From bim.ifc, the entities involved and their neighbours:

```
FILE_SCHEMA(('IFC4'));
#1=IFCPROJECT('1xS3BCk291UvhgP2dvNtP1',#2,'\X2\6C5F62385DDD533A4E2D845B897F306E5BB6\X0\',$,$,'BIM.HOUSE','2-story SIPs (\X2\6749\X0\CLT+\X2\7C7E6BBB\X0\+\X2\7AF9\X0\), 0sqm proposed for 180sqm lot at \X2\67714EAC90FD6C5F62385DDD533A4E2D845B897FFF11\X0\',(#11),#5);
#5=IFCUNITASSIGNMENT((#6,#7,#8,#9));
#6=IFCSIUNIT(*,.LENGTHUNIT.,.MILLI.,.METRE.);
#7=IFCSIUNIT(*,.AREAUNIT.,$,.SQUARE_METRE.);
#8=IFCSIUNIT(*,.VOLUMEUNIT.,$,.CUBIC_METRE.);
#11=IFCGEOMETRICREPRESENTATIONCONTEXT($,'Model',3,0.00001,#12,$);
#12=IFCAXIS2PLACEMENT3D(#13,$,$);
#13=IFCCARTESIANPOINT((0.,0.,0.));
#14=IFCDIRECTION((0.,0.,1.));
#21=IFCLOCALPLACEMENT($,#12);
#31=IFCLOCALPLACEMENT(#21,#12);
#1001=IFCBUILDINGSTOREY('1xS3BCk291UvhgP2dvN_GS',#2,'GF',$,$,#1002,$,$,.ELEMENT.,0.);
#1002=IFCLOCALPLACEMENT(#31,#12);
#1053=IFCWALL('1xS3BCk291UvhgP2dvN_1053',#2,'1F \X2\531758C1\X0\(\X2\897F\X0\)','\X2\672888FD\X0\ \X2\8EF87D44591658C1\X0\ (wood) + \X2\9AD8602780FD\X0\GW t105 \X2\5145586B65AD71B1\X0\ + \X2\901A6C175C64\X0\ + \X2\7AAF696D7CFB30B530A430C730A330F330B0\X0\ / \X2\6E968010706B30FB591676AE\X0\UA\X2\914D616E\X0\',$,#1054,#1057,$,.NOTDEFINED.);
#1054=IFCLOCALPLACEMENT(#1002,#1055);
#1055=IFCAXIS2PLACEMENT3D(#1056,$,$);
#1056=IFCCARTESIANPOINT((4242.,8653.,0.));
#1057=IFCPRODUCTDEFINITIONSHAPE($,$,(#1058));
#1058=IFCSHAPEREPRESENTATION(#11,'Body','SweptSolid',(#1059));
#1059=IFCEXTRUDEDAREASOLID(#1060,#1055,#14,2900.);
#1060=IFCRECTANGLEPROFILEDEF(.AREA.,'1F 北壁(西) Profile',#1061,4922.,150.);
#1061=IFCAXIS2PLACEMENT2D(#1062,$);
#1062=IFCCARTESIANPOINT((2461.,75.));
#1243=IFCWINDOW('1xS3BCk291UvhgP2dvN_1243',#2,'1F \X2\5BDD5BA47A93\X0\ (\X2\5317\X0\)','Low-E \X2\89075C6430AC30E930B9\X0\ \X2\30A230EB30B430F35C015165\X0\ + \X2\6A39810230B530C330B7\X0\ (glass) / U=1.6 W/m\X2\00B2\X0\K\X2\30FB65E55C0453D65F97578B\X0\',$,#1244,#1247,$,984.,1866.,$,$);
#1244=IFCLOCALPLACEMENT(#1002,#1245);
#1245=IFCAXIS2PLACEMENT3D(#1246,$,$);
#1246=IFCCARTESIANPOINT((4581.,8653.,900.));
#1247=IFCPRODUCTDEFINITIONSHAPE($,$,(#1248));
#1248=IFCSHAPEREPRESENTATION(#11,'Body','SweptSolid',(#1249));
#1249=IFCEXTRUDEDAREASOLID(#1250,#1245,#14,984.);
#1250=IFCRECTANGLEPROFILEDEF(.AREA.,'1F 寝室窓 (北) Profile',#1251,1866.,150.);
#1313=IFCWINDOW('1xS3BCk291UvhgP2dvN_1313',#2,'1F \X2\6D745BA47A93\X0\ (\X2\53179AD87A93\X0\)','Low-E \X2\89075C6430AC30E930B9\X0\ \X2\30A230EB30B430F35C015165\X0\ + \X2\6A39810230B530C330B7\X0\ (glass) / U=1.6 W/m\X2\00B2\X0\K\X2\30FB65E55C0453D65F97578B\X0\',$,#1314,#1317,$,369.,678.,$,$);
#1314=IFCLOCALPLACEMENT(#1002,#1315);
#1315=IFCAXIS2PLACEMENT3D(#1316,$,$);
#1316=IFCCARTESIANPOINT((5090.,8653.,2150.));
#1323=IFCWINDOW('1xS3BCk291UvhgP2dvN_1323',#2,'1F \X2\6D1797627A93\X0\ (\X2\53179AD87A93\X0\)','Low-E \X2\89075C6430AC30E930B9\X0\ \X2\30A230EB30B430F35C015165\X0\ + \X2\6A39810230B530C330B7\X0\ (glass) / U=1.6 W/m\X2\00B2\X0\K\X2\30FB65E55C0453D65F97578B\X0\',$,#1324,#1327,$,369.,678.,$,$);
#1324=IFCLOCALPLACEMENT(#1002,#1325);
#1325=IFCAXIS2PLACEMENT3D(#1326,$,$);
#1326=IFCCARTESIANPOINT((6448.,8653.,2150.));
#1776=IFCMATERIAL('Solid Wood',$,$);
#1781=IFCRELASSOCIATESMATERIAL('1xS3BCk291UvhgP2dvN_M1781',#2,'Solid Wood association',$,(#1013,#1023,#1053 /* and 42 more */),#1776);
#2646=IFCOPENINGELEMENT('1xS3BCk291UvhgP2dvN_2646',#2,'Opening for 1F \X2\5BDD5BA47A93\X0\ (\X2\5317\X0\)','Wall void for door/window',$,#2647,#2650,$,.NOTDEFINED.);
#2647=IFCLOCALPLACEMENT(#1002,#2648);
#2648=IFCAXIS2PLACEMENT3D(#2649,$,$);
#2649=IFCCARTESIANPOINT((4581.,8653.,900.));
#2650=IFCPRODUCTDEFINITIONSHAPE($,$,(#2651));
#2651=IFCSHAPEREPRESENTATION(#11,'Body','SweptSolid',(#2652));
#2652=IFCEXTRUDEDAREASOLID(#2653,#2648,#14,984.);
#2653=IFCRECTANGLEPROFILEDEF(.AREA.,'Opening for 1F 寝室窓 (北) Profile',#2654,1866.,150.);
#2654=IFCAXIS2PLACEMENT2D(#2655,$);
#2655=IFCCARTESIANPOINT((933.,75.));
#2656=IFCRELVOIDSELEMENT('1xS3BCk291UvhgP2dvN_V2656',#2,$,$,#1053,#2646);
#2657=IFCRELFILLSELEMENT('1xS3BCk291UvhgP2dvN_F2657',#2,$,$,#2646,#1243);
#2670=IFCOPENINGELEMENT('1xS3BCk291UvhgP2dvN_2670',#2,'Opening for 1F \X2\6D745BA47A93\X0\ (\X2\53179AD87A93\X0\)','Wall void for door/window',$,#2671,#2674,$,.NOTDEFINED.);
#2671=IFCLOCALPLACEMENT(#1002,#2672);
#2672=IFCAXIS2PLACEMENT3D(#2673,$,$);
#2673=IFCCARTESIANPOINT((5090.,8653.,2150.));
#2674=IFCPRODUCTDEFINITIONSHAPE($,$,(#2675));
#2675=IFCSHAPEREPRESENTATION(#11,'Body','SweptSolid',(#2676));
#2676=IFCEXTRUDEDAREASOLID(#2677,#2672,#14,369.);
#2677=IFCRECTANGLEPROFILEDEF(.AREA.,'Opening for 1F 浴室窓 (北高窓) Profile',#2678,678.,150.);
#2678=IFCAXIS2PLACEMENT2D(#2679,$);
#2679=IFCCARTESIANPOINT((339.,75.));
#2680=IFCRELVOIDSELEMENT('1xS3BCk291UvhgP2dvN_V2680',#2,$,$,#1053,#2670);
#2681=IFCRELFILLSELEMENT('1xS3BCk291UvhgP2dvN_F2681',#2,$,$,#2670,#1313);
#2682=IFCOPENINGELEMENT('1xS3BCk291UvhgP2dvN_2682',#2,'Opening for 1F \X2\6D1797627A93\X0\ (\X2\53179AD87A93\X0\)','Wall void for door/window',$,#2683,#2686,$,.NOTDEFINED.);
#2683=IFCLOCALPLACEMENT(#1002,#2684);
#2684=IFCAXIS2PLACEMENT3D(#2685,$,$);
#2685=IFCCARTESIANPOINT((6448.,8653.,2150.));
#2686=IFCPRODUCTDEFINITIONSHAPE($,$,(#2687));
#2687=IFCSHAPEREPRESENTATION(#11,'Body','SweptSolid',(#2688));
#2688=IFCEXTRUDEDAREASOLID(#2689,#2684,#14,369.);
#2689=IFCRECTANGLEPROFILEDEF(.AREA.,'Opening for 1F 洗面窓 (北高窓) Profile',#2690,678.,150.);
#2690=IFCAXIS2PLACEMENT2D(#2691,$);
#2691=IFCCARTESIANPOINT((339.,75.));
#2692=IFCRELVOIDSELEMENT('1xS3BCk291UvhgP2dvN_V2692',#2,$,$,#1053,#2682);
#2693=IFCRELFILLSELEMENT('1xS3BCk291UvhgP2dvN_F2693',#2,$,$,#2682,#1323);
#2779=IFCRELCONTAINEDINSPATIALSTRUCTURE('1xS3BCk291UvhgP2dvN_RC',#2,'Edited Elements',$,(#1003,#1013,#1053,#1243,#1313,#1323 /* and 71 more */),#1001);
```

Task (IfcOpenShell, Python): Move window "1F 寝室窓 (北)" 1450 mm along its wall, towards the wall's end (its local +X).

```python
import ifcopenshell
import ifcopenshell.api.geometry
import ifcopenshell.util.placement
import ifcopenshell.util.unit

model = ifcopenshell.open("bim.ifc")
unit_scale = ifcopenshell.util.unit.calculate_unit_scale(model)

window = model.by_guid("1xS3BCk291UvhgP2dvN_1243")
opening = window.FillsVoids[0].RelatingOpeningElement
wall = opening.VoidsElements[0].RelatingBuildingElement

wall_matrix = ifcopenshell.util.placement.get_local_placement(wall.ObjectPlacement)
shift = wall_matrix[:3, 0] * 1.45 / unit_scale
before = ifcopenshell.util.placement.get_local_placement(window.ObjectPlacement)[:3, 3].copy()

# The window is not placed relative to its opening, so move both.
for product in (opening, window):
    matrix = ifcopenshell.util.placement.get_local_placement(product.ObjectPlacement)
    matrix[:3, 3] += shift
    ifcopenshell.api.geometry.edit_object_placement(model, product=product, matrix=matrix, is_si=False)

after = ifcopenshell.util.placement.get_local_placement(window.ObjectPlacement)[:3, 3]
print("window moved by", (after - before).round(3) + 0.0)

model.write("bim_rev.ifc")
```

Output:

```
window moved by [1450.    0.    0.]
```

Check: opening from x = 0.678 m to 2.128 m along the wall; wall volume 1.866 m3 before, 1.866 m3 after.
